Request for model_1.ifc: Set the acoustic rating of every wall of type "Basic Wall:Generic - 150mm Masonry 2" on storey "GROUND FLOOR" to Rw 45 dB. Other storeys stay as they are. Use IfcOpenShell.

First a look at what the model holds.

```python
import ifcopenshell
import ifcopenshell.util.element

model = ifcopenshell.open("model_1.ifc")
print(model.schema)
storey = next(s for s in model.by_type("IfcBuildingStorey") if s.Name == "GROUND FLOOR")
walls = [e for e in ifcopenshell.util.element.get_decomposition(storey) if e.is_a("IfcWall")]
seen = {}
for e in walls:
    element_type = ifcopenshell.util.element.get_type(e)
    key = (element_type.Name if element_type != e and element_type else None, ifcopenshell.util.element.get_pset(e, "Pset_WallCommon", "AcousticRating"))
    seen[key] = seen.get(key, 0) + 1
for (name, value), count in sorted(seen.items(), key=str):
    print(count, "x", name, "|", value)
```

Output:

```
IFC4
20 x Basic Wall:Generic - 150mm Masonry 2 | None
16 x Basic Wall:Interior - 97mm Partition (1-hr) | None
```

```python
import ifcopenshell
import ifcopenshell.api.pset
import ifcopenshell.util.element

model = ifcopenshell.open("model_1.ifc")

storey = next(s for s in model.by_type("IfcBuildingStorey") if s.Name == "GROUND FLOOR")
walls = [e for e in ifcopenshell.util.element.get_decomposition(storey) if e.is_a("IfcWall")]

count = 0
for e in walls:
    element_type = ifcopenshell.util.element.get_type(e)
    if element_type in (None, e) or element_type.Name != "Basic Wall:Generic - 150mm Masonry 2":
        continue
    # add_pset returns the element's existing set when there is one.
    pset = ifcopenshell.api.pset.add_pset(model, product=e, name="Pset_WallCommon")
    ifcopenshell.api.pset.edit_pset(model, pset=pset, properties={"AcousticRating": "Rw 45 dB"})
    count += 1

print(count, "walls updated")

model.write("model_1_v2.ifc")
```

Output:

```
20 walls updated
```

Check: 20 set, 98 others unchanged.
